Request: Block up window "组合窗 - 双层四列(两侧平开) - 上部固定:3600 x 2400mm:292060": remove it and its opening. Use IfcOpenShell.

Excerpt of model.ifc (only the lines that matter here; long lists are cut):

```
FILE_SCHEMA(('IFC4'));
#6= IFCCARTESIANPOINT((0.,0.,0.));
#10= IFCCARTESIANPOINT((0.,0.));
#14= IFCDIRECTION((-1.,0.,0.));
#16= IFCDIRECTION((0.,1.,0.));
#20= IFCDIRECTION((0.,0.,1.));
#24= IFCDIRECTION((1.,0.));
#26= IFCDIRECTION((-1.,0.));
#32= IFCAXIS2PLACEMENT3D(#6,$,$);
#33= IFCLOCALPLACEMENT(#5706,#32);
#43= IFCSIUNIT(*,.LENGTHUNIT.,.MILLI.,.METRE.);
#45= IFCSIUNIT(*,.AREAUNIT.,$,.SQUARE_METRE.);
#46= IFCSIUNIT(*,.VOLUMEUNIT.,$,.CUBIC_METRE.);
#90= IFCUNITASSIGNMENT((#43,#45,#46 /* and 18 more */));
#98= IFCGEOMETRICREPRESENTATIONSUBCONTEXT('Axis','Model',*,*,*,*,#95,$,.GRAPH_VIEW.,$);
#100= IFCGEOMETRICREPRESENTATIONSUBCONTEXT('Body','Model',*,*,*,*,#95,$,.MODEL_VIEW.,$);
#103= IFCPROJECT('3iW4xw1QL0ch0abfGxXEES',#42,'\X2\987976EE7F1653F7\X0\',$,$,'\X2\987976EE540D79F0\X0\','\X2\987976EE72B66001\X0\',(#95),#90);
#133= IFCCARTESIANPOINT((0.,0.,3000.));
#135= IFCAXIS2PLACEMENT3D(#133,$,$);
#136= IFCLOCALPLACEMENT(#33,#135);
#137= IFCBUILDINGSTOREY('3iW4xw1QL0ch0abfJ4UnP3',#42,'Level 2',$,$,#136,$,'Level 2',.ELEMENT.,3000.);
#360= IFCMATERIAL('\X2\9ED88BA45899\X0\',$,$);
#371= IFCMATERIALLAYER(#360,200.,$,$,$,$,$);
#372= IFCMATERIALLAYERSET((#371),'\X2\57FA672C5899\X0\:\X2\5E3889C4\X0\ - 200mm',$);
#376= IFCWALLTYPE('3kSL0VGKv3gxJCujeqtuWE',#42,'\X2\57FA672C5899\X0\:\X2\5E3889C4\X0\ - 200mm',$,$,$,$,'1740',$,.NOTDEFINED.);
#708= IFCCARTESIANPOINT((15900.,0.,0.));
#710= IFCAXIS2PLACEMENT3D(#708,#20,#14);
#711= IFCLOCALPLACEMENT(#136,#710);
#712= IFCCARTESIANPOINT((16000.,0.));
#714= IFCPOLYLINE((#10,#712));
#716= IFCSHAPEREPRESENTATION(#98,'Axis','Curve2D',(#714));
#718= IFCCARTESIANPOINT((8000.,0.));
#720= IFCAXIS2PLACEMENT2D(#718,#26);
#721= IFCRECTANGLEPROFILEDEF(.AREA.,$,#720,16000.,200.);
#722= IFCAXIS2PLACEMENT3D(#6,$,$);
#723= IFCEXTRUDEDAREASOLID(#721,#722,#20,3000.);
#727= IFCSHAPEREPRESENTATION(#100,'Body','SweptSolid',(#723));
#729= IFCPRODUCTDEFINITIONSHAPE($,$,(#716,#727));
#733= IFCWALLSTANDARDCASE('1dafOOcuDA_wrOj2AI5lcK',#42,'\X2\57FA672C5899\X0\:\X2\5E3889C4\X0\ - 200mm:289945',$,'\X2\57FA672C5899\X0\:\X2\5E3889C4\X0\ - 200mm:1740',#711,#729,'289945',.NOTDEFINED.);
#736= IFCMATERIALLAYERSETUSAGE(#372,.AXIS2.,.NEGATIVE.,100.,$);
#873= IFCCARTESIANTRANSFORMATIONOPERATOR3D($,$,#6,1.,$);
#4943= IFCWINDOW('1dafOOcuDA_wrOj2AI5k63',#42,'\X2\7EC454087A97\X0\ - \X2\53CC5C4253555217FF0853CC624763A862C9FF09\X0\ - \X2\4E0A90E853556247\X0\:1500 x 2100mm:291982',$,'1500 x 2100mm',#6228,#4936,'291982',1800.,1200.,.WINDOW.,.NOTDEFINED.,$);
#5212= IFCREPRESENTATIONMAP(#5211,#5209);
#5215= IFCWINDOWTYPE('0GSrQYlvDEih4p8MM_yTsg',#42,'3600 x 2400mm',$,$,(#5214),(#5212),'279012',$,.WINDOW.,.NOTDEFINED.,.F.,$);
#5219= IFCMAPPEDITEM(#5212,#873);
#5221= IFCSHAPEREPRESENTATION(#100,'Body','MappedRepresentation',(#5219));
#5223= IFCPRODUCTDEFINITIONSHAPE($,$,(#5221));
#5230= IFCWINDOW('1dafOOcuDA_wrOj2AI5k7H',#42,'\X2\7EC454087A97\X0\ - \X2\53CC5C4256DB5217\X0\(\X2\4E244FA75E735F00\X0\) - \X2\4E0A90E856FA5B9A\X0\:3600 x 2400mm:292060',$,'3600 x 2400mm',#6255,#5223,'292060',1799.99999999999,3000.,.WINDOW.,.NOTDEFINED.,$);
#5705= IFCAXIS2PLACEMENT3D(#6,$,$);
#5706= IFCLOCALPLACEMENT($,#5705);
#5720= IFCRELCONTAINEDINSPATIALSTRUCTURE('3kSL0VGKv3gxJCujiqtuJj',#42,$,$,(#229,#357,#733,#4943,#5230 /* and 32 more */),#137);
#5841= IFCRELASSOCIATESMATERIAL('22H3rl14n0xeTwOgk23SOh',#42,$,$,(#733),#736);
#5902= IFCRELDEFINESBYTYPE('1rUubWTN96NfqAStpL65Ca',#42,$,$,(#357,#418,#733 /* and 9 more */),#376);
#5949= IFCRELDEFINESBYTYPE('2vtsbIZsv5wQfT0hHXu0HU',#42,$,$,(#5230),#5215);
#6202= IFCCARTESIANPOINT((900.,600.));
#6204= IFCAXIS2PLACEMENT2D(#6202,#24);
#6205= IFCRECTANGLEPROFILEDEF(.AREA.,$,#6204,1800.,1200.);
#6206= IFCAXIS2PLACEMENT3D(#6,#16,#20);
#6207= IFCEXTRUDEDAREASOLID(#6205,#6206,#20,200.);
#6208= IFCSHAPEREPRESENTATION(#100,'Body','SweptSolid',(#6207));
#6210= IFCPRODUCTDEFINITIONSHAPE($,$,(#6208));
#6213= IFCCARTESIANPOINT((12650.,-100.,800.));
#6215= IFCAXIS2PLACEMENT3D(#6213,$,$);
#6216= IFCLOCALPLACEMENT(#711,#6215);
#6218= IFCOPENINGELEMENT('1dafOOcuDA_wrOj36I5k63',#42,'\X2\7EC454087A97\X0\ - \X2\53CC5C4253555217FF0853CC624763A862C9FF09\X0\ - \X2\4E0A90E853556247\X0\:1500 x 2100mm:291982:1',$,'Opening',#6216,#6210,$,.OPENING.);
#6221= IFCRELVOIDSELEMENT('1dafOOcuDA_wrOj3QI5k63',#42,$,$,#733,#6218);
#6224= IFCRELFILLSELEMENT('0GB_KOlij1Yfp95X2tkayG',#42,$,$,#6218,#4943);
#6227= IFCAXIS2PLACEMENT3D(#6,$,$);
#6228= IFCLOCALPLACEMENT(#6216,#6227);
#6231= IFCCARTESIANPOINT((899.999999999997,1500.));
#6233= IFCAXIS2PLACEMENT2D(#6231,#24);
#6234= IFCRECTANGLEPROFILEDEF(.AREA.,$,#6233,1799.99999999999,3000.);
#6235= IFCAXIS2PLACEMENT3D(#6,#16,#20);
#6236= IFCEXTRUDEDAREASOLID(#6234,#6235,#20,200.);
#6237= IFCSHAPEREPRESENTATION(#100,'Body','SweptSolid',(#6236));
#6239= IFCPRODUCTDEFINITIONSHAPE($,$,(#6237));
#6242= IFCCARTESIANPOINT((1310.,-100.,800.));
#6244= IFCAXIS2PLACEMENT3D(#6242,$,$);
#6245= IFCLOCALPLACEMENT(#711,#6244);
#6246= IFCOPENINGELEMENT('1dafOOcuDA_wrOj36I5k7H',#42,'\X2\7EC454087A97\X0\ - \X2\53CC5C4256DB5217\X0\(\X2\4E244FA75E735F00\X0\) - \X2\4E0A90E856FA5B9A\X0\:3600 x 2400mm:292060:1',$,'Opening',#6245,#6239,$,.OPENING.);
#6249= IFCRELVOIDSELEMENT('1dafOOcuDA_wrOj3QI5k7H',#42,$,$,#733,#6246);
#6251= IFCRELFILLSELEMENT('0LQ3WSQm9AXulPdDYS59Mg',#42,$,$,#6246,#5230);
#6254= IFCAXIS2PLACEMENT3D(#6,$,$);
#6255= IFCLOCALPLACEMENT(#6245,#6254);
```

```python
import ifcopenshell
import ifcopenshell.api.feature
import ifcopenshell.api.root
import ifcopenshell.geom
import ifcopenshell.util.shape

model = ifcopenshell.open("model.ifc")
settings = ifcopenshell.geom.settings()


def volume(element):
    """Net volume in cubic metres, openings subtracted."""
    shape = ifcopenshell.geom.create_shape(settings, element)
    return ifcopenshell.util.shape.get_volume(shape.geometry)


window = model.by_id(5230)
opening = window.FillsVoids[0].RelatingOpeningElement
wall = opening.VoidsElements[0].RelatingBuildingElement
before = volume(wall)

ifcopenshell.api.root.remove_product(model, product=window)
ifcopenshell.api.feature.remove_feature(model, feature=opening)

after = volume(wall)

print(f"wall volume {before:.3f} -> {after:.3f} m3")

model.write("model_rev.ifc")
```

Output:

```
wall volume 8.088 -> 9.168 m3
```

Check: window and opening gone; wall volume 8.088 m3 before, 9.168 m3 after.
